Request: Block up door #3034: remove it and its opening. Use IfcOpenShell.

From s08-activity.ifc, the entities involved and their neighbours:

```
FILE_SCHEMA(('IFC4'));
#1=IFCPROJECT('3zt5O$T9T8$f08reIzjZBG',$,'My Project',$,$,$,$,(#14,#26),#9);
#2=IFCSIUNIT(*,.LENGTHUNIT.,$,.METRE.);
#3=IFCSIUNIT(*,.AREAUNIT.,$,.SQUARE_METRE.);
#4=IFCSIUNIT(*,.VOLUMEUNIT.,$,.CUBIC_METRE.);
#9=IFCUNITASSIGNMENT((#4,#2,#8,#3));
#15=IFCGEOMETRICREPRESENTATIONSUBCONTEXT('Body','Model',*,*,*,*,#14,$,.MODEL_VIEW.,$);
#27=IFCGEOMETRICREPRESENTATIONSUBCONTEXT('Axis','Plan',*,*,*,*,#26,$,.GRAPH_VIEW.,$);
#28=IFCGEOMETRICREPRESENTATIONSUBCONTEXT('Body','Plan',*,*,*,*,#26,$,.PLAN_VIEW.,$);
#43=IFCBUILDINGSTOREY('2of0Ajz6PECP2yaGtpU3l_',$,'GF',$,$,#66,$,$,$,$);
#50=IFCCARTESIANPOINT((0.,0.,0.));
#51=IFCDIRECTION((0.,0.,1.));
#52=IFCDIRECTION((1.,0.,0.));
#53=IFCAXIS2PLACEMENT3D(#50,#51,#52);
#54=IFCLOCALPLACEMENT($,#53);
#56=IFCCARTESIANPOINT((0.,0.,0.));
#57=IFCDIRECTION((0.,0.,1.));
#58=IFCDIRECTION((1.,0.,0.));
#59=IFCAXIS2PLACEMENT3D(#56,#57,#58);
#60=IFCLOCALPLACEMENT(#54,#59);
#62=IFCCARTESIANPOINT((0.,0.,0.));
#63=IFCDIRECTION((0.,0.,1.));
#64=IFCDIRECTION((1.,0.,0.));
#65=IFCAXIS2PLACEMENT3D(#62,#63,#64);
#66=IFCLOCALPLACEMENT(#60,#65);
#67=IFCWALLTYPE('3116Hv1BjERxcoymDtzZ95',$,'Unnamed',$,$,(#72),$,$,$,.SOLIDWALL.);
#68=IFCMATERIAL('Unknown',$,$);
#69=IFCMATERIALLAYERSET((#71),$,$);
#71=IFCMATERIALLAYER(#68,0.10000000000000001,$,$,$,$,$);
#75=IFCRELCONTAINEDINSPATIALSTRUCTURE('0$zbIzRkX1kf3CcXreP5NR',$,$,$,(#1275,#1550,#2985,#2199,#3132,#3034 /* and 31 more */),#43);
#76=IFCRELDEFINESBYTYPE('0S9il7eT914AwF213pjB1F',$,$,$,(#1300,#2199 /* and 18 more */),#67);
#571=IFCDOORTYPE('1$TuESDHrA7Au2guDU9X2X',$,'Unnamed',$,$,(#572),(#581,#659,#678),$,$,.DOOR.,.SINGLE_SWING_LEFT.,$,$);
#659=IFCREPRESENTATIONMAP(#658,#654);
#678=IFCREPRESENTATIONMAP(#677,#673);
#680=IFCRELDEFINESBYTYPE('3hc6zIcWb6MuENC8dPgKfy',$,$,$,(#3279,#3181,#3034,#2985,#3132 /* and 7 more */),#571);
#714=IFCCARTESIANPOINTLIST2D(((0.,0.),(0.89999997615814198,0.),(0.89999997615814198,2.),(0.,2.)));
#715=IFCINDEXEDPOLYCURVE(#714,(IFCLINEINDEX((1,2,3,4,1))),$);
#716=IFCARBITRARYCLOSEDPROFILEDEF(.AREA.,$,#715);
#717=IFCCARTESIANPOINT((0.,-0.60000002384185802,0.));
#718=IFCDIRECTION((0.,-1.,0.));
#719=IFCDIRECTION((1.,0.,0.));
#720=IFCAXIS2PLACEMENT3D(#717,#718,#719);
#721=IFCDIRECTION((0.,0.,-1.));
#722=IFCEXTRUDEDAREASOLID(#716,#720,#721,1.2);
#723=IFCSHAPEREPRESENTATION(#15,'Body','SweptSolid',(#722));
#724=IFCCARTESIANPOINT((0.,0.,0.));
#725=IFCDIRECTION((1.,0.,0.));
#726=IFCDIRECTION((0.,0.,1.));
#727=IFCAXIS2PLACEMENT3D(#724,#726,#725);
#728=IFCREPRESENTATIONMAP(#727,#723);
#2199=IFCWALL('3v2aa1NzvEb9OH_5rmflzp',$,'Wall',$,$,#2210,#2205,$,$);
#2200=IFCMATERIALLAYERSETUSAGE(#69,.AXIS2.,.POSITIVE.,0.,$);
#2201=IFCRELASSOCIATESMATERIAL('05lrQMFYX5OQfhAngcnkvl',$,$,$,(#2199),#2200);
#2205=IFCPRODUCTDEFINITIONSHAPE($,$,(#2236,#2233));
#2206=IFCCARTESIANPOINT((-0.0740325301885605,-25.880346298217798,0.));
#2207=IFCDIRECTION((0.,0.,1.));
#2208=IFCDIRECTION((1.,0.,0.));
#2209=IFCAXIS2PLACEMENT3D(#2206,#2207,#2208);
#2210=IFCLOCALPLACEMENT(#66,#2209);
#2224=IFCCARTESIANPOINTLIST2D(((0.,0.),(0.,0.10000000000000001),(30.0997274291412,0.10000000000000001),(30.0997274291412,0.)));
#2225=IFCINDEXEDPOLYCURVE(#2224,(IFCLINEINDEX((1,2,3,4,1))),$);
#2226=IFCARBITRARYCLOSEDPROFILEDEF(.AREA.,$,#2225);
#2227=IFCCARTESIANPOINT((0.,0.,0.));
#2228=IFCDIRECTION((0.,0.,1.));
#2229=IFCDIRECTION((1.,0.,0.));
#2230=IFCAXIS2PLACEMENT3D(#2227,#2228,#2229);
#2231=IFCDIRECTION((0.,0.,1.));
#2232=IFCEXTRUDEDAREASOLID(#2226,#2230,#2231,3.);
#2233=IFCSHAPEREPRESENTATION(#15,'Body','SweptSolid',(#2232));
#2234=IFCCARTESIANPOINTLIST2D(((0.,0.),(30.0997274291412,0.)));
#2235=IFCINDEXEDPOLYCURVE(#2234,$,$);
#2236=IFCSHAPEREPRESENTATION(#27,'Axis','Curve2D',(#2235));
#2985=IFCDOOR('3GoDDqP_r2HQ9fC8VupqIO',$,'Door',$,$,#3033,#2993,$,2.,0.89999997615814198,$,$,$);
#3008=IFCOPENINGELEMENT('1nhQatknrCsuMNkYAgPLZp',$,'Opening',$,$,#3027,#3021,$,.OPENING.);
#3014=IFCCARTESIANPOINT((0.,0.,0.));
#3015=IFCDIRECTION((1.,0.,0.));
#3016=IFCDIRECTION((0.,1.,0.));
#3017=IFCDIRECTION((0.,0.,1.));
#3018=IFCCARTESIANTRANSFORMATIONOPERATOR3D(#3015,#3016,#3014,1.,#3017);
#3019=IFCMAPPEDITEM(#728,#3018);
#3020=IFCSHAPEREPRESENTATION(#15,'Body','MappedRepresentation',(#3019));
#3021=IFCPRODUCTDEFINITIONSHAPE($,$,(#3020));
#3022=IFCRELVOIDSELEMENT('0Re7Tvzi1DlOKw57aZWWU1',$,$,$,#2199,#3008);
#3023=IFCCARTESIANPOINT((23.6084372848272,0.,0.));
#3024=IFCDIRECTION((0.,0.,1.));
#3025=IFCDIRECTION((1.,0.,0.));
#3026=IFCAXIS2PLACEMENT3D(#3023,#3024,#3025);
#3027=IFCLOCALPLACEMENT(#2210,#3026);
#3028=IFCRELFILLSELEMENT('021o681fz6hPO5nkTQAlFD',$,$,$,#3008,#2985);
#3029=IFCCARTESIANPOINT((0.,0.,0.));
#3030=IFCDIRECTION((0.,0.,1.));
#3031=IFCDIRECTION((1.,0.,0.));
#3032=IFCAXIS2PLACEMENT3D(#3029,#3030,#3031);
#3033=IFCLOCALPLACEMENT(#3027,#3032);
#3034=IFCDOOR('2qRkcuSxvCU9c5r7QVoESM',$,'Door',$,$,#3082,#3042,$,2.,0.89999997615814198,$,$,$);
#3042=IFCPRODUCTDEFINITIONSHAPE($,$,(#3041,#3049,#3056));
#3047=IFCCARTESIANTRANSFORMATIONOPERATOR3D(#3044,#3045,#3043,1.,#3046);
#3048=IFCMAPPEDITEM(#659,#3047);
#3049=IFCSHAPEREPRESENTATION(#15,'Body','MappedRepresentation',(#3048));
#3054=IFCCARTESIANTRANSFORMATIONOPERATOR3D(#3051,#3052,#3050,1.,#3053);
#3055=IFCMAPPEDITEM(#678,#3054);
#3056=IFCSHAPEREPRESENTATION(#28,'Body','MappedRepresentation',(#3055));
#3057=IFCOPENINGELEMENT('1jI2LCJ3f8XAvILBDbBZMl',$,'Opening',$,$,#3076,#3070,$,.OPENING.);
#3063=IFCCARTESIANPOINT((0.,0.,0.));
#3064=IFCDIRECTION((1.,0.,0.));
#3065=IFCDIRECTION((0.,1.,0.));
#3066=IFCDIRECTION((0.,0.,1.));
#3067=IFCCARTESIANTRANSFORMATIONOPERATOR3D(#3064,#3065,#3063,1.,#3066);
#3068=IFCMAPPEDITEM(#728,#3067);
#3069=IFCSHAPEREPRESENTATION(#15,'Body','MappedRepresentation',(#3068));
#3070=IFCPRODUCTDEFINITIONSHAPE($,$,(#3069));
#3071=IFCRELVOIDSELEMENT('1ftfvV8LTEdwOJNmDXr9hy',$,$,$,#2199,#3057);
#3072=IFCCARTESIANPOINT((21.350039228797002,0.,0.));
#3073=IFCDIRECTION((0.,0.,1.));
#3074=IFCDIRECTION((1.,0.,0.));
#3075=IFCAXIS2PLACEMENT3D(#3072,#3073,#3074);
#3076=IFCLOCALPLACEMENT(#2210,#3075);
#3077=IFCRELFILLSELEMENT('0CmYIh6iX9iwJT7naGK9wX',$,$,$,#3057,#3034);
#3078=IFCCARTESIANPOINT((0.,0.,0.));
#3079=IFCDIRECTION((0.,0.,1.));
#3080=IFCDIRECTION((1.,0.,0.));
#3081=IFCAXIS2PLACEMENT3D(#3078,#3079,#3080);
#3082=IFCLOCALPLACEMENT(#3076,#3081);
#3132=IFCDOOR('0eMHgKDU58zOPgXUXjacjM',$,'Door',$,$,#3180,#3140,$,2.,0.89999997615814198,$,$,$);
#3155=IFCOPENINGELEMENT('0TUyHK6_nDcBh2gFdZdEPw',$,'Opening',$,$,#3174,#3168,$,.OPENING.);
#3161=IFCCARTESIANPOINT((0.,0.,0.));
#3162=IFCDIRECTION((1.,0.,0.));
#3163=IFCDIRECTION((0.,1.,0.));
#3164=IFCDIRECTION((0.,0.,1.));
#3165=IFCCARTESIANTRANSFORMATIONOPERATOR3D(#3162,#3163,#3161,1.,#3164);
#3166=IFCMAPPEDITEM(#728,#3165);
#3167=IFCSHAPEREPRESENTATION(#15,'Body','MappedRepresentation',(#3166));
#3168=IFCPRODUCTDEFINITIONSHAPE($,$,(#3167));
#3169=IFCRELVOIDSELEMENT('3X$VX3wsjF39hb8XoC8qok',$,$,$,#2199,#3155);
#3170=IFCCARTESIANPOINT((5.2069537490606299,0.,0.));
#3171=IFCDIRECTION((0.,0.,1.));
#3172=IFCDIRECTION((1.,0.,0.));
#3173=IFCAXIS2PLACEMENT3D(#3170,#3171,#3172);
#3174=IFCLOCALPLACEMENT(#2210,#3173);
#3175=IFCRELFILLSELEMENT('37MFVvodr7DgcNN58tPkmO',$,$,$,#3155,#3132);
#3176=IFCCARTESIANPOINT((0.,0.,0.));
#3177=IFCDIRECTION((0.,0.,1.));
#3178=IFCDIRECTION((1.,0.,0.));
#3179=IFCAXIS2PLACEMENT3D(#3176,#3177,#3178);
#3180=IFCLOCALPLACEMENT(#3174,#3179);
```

```python
import ifcopenshell
import ifcopenshell.api.feature
import ifcopenshell.api.root
import ifcopenshell.geom
import ifcopenshell.util.shape

model = ifcopenshell.open("s08-activity.ifc")
settings = ifcopenshell.geom.settings()


def volume(element):
    """Net volume in cubic metres, openings subtracted."""
    shape = ifcopenshell.geom.create_shape(settings, element)
    return ifcopenshell.util.shape.get_volume(shape.geometry)


door = model.by_guid("2qRkcuSxvCU9c5r7QVoESM")
opening = door.FillsVoids[0].RelatingOpeningElement
wall = opening.VoidsElements[0].RelatingBuildingElement
before = volume(wall)

ifcopenshell.api.root.remove_product(model, product=door)
ifcopenshell.api.feature.remove_feature(model, feature=opening)

after = volume(wall)

print(f"wall volume {before:.3f} -> {after:.3f} m3")

model.write("s08-activity-out.ifc")
```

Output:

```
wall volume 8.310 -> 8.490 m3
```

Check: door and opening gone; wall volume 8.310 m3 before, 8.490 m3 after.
